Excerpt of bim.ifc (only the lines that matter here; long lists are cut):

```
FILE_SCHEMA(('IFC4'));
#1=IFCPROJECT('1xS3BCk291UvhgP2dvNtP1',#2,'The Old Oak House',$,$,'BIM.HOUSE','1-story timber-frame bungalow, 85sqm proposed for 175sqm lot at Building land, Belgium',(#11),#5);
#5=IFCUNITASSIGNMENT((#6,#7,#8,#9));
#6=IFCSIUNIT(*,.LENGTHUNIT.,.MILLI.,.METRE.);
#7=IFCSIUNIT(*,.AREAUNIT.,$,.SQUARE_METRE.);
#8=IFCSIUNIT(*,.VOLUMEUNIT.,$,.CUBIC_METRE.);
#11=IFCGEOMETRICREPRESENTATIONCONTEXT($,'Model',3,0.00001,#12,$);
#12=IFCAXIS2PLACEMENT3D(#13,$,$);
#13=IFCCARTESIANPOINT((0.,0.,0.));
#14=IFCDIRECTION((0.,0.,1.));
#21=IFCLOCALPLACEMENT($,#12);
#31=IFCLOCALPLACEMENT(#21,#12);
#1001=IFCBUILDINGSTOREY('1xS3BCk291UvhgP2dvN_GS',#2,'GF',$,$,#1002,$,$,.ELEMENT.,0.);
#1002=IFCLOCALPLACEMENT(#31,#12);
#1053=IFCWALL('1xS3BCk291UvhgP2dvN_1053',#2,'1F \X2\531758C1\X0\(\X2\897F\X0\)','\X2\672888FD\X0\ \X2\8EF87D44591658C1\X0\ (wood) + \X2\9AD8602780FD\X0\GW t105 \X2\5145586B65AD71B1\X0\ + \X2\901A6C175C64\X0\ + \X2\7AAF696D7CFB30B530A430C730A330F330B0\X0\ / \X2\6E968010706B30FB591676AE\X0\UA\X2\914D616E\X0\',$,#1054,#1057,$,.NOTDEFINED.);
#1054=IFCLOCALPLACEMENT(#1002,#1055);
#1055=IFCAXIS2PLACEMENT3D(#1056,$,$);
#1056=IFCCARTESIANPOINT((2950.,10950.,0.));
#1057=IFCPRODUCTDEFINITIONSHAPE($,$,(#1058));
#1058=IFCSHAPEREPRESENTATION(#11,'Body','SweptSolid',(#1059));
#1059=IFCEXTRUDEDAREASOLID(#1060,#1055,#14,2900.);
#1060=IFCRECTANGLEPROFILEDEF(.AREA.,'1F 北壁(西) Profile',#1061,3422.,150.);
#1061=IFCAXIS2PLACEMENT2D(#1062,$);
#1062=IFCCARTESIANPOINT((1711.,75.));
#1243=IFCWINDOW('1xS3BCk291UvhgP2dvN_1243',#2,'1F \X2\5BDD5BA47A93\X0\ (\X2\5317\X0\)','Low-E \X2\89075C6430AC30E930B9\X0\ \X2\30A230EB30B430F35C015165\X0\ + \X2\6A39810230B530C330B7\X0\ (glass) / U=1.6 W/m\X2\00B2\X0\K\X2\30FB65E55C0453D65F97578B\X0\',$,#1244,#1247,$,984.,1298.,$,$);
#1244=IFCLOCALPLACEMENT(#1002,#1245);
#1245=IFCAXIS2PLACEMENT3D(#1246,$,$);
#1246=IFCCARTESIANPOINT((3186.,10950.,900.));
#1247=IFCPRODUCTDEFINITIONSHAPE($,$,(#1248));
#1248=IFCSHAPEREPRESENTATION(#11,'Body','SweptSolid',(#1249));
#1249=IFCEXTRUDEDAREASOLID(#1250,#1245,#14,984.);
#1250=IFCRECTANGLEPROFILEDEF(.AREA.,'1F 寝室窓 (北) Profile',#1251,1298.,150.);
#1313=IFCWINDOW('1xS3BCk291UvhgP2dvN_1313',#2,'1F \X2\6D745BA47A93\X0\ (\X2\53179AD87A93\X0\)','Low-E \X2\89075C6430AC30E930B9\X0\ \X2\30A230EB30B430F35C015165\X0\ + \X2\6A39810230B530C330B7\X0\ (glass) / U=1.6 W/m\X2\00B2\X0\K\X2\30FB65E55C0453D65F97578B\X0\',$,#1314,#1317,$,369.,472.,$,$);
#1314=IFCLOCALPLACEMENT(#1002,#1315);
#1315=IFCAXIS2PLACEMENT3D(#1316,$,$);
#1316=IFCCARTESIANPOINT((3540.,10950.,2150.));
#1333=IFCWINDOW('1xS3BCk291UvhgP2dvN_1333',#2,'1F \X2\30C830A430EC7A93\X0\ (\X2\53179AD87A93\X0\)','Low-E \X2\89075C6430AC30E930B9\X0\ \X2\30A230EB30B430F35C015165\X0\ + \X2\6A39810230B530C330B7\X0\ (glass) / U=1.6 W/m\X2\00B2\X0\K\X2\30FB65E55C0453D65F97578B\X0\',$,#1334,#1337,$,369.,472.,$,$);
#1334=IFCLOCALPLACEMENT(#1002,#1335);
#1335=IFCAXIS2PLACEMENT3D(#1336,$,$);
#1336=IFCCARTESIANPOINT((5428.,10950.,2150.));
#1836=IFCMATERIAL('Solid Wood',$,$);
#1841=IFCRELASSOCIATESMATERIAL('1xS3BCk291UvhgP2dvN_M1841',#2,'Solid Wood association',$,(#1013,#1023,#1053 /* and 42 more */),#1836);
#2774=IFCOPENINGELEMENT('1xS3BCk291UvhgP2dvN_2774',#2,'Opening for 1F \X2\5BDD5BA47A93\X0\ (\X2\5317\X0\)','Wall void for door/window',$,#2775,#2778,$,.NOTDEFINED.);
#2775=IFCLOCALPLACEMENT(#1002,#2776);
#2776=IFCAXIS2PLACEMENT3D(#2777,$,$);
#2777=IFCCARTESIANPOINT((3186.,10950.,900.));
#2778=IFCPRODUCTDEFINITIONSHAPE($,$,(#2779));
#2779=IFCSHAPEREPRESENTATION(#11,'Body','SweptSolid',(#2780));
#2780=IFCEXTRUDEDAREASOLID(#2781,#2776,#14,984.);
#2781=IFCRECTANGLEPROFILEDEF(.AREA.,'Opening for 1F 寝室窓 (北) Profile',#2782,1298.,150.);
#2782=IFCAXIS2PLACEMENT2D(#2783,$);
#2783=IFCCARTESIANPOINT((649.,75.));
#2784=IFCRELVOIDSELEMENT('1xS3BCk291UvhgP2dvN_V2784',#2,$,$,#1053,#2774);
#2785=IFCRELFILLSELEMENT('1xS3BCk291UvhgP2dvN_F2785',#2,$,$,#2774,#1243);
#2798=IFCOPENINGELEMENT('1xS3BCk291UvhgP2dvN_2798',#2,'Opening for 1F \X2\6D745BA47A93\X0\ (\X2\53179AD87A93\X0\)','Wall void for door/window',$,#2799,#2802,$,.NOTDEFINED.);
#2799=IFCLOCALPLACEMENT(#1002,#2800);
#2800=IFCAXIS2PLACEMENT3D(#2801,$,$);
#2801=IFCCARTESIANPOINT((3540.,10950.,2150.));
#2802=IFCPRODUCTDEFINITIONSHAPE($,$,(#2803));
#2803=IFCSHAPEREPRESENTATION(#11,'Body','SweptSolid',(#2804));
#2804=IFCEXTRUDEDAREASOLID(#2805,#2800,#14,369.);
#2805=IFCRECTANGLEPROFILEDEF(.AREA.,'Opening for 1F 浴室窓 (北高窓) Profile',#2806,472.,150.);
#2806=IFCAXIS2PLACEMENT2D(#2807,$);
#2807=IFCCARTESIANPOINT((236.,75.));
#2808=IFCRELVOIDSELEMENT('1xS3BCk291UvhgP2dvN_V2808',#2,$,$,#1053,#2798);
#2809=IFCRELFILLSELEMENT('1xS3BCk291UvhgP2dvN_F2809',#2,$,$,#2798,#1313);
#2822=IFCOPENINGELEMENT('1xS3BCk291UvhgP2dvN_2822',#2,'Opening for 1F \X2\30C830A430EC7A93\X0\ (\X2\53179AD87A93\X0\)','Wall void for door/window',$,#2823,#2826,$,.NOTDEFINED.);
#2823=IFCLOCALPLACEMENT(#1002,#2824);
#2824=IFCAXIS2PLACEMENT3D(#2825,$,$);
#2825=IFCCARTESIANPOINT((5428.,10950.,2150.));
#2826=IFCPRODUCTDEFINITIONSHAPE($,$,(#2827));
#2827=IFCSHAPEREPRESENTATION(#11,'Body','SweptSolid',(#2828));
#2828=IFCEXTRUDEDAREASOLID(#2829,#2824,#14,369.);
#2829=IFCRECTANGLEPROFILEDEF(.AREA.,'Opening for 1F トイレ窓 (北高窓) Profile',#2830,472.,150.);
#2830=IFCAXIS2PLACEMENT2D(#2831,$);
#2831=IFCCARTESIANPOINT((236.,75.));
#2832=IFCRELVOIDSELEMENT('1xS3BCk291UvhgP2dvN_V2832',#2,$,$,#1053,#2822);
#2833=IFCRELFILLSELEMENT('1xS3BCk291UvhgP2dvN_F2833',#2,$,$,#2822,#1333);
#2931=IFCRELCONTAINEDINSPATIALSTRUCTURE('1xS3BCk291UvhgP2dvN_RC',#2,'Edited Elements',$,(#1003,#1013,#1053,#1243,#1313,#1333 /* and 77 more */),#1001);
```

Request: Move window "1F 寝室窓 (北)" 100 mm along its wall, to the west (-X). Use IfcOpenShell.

```python
import ifcopenshell
import ifcopenshell.api.geometry
import ifcopenshell.util.placement

model = ifcopenshell.open("bim.ifc")

window = model.by_id(1243)
opening = window.FillsVoids[0].RelatingOpeningElement
wall = opening.VoidsElements[0].RelatingBuildingElement

wall_matrix = ifcopenshell.util.placement.get_local_placement(wall.ObjectPlacement)
shift = wall_matrix[:3, 0] * -100.0
before = ifcopenshell.util.placement.get_local_placement(window.ObjectPlacement)[:3, 3].copy()

# The window is not placed relative to its opening, so move both.
for product in (opening, window):
    matrix = ifcopenshell.util.placement.get_local_placement(product.ObjectPlacement)
    matrix[:3, 3] += shift
    ifcopenshell.api.geometry.edit_object_placement(model, product=product, matrix=matrix, is_si=False)

after = ifcopenshell.util.placement.get_local_placement(window.ObjectPlacement)[:3, 3]
print("window moved by", (after - before).round(3) + 0.0)

model.write("bim_v2.ifc")
```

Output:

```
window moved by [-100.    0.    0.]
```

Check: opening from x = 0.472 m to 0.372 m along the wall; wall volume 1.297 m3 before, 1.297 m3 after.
